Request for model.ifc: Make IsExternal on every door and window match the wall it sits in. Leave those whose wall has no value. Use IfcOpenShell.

First a look at what the model holds.

```python
import ifcopenshell
import ifcopenshell.util.element

model = ifcopenshell.open("model.ifc")
print(model.schema)
seen = {}
for e in model.by_type("IfcDoor") + model.by_type("IfcWindow"):
    if not e.FillsVoids:
        continue
    host = e.FillsVoids[0].RelatingOpeningElement.VoidsElements[0].RelatingBuildingElement
    own = ifcopenshell.util.element.get_pset(e, f"Pset_{e.is_a()[3:].removesuffix('StandardCase')}Common", "IsExternal")
    wall = ifcopenshell.util.element.get_pset(host, "Pset_WallCommon", "IsExternal")
    seen[e.is_a(), own, wall] = seen.get((e.is_a(), own, wall), 0) + 1
for (cls, own, wall), count in sorted(seen.items(), key=str):
    print(count, cls, "IsExternal:", own, "| host wall:", wall)
```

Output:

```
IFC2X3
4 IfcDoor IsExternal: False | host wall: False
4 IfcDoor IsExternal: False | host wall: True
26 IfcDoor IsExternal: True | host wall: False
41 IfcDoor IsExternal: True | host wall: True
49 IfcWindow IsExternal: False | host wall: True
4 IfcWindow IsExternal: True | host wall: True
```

```python
import ifcopenshell
import ifcopenshell.api.pset
import ifcopenshell.util.element

model = ifcopenshell.open("model.ifc")

count = 0
for ifc_class, pset_name in (("IfcDoor", "Pset_DoorCommon"), ("IfcWindow", "Pset_WindowCommon")):
    for e in model.by_type(ifc_class):
        if not e.FillsVoids:
            continue
        host = e.FillsVoids[0].RelatingOpeningElement.VoidsElements[0].RelatingBuildingElement
        external = ifcopenshell.util.element.get_pset(host, "Pset_WallCommon", "IsExternal")
        if external is None or ifcopenshell.util.element.get_pset(e, pset_name, "IsExternal") == external:
            continue
        pset = ifcopenshell.api.pset.add_pset(model, product=e, name=pset_name)
        ifcopenshell.api.pset.edit_pset(model, pset=pset, properties={"IsExternal": external})
        count += 1

print(count, "updated")

model.write("model_v2.ifc")
```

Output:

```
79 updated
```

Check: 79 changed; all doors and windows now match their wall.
